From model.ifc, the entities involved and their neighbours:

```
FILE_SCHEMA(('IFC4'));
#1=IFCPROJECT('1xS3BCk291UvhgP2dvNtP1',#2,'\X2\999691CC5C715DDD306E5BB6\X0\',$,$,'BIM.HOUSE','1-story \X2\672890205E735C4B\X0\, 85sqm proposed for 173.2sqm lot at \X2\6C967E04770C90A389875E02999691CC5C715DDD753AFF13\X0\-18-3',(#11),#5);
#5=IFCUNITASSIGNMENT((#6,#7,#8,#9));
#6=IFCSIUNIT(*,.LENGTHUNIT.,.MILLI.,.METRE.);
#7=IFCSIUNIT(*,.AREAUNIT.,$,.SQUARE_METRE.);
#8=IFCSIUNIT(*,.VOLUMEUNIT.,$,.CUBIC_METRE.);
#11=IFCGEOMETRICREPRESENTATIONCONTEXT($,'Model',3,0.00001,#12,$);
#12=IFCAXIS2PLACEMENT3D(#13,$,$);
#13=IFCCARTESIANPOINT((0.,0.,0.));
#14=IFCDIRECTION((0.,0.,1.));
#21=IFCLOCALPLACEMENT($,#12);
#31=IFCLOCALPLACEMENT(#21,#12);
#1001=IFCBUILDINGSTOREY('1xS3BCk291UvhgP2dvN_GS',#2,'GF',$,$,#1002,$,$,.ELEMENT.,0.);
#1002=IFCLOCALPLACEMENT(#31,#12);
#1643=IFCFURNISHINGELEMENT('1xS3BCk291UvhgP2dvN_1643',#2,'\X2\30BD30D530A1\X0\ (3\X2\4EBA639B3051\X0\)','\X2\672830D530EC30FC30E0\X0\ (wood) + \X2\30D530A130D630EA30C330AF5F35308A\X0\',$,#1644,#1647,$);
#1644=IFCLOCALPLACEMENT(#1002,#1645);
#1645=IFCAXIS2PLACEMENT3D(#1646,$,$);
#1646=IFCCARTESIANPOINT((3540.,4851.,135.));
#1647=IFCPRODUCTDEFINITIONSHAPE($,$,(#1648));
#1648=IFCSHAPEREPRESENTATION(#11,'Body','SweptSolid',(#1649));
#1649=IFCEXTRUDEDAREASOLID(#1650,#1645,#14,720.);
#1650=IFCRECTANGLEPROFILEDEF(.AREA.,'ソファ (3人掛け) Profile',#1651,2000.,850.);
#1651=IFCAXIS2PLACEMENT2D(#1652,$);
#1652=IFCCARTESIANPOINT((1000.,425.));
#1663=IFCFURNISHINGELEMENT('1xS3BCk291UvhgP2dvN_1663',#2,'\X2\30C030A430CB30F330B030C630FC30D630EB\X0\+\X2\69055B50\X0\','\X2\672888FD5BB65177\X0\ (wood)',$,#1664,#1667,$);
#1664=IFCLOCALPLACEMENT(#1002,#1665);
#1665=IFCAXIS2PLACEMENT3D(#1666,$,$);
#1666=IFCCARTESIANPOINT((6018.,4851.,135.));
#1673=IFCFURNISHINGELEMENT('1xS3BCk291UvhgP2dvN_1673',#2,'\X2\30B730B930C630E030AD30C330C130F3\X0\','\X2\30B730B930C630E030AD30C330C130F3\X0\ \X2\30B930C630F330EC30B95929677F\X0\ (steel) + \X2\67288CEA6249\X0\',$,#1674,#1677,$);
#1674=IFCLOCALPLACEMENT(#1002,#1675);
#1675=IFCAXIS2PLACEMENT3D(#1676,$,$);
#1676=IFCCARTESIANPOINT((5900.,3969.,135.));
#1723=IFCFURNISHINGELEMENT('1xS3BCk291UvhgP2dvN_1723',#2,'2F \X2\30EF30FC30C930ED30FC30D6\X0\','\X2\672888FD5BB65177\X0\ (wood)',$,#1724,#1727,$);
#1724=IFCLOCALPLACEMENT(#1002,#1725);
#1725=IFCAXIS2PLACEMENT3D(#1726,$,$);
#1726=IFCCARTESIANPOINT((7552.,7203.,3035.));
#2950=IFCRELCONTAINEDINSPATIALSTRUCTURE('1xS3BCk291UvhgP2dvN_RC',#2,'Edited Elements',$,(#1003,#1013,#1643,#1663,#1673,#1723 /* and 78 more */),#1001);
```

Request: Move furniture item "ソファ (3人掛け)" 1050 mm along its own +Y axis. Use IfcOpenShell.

```python
import ifcopenshell
import ifcopenshell.api.geometry
import ifcopenshell.util.placement
import ifcopenshell.util.unit

model = ifcopenshell.open("model.ifc")
unit_scale = ifcopenshell.util.unit.calculate_unit_scale(model)

item = model.by_id(1643)
matrix = ifcopenshell.util.placement.get_local_placement(item.ObjectPlacement)
matrix[:3, 3] += matrix[:3, 1] * 1.05 / unit_scale
ifcopenshell.api.geometry.edit_object_placement(model, product=item, matrix=matrix, is_si=False)

print(ifcopenshell.util.placement.get_local_placement(item.ObjectPlacement).round(3) + 0.0)

model.write("model_edited.ifc")
```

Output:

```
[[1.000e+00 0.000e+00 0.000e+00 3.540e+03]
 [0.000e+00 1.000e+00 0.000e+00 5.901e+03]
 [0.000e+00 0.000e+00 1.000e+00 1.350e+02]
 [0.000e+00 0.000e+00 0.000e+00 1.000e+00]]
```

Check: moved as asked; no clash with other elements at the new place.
